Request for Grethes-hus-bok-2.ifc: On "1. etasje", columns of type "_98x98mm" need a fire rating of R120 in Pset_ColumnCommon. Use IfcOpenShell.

First a look at what the model holds.

```python
import ifcopenshell
import ifcopenshell.util.element

model = ifcopenshell.open("Grethes-hus-bok-2.ifc")
print(model.schema)
storey = next(s for s in model.by_type("IfcBuildingStorey") if s.Name == "1. etasje")
columns = [e for e in ifcopenshell.util.element.get_decomposition(storey) if e.is_a("IfcColumn")]
seen = {}
for e in columns:
    element_type = ifcopenshell.util.element.get_type(e)
    key = (element_type.Name if element_type != e and element_type else None, ifcopenshell.util.element.get_pset(e, "Pset_ColumnCommon", "FireRating"))
    seen[key] = seen.get(key, 0) + 1
for (name, value), count in sorted(seen.items(), key=str):
    print(count, "x", name, "|", value)
```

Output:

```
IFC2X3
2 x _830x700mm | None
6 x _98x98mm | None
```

```python
import ifcopenshell
import ifcopenshell.api.pset
import ifcopenshell.util.element

model = ifcopenshell.open("Grethes-hus-bok-2.ifc")

storey = next(s for s in model.by_type("IfcBuildingStorey") if s.Name == "1. etasje")
columns = [e for e in ifcopenshell.util.element.get_decomposition(storey) if e.is_a("IfcColumn")]

count = 0
for e in columns:
    element_type = ifcopenshell.util.element.get_type(e)
    if element_type in (None, e) or element_type.Name != "_98x98mm":
        continue
    # add_pset returns the element's existing set when there is one.
    pset = ifcopenshell.api.pset.add_pset(model, product=e, name="Pset_ColumnCommon")
    ifcopenshell.api.pset.edit_pset(model, pset=pset, properties={"FireRating": "R120"})
    count += 1

print(count, "columns updated")

model.write("Grethes-hus-bok-2-out.ifc")
```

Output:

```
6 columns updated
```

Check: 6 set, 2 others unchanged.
